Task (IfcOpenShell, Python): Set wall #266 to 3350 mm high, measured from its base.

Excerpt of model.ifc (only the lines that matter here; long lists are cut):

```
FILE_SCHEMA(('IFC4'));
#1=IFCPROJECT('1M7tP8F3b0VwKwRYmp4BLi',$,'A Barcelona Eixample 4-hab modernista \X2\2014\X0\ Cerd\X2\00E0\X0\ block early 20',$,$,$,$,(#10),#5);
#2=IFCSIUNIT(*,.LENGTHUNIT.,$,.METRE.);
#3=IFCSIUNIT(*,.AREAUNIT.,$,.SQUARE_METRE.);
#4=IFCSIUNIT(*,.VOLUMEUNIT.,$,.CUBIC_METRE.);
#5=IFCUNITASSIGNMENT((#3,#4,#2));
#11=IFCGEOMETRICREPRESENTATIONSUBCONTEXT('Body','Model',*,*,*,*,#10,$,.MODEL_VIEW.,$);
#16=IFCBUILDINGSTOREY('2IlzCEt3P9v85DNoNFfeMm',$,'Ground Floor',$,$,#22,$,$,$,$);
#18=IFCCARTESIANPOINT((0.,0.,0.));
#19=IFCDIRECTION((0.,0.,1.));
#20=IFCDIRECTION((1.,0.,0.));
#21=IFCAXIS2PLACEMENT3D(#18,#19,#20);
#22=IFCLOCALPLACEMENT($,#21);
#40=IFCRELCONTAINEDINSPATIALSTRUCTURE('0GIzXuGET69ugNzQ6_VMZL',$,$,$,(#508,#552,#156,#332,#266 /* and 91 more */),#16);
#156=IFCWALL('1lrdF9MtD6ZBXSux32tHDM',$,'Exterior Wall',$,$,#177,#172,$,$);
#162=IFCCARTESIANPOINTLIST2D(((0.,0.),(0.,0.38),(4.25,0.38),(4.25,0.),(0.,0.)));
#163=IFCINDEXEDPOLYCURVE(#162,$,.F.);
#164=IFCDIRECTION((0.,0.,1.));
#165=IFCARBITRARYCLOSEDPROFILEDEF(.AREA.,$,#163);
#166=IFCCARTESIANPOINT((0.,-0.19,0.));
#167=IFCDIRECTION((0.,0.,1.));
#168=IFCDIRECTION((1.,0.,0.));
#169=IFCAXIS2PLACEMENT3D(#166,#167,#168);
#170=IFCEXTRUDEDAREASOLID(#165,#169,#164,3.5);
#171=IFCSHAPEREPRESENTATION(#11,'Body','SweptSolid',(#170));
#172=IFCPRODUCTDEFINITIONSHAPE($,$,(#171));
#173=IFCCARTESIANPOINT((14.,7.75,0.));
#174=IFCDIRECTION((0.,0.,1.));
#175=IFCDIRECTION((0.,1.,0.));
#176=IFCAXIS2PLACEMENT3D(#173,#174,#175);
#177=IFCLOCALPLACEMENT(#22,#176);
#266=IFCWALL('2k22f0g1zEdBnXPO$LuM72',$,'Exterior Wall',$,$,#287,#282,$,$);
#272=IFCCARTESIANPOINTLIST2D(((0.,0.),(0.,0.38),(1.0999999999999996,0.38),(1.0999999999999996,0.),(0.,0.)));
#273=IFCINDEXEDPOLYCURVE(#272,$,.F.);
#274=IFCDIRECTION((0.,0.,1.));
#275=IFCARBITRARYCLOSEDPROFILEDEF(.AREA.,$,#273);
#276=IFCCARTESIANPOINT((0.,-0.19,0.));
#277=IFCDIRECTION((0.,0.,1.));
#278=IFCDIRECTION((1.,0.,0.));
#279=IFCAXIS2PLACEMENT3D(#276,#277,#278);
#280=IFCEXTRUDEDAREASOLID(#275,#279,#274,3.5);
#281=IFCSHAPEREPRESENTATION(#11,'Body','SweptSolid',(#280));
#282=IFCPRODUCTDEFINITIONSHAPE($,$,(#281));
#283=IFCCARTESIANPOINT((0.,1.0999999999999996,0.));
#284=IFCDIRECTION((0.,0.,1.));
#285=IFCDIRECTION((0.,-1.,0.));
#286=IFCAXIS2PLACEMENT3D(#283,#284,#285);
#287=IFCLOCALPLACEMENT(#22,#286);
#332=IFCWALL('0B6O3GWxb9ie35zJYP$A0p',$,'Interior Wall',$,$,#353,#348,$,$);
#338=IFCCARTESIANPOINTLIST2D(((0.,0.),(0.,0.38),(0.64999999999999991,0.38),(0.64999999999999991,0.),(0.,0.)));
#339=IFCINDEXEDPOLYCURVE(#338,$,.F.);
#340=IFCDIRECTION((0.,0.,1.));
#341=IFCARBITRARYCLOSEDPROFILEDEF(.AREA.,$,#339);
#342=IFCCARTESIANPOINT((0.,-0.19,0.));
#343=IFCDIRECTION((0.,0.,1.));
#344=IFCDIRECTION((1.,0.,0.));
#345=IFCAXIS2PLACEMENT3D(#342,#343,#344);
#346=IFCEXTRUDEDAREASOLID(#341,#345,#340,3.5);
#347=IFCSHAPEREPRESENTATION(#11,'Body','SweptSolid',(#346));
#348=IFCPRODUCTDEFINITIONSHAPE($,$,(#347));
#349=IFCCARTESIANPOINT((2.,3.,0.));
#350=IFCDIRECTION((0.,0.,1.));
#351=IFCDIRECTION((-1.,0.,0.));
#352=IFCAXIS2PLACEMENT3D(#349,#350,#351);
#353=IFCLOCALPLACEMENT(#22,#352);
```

```python
import ifcopenshell
import ifcopenshell.geom
import ifcopenshell.util.representation
import ifcopenshell.util.shape
import ifcopenshell.util.unit

model = ifcopenshell.open("model.ifc")
unit_scale = ifcopenshell.util.unit.calculate_unit_scale(model)
settings = ifcopenshell.geom.settings()


def volume(element):
    """Net volume in cubic metres, openings subtracted."""
    shape = ifcopenshell.geom.create_shape(settings, element)
    return ifcopenshell.util.shape.get_volume(shape.geometry)


wall = model.by_guid("2k22f0g1zEdBnXPO$LuM72")
before = volume(wall)

body = ifcopenshell.util.representation.get_representation(wall, "Model", "Body")
solid = body.Items[0]
old_height = solid.Depth
solid.Depth = 3.35 / unit_scale
after = volume(wall)

print(f"height {old_height:g} -> {solid.Depth:g}, volume {before:.3f} -> {after:.3f} m3")

model.write("model_rev.ifc")
```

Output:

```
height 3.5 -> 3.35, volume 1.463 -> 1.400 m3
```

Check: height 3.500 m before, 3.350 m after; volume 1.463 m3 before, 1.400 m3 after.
